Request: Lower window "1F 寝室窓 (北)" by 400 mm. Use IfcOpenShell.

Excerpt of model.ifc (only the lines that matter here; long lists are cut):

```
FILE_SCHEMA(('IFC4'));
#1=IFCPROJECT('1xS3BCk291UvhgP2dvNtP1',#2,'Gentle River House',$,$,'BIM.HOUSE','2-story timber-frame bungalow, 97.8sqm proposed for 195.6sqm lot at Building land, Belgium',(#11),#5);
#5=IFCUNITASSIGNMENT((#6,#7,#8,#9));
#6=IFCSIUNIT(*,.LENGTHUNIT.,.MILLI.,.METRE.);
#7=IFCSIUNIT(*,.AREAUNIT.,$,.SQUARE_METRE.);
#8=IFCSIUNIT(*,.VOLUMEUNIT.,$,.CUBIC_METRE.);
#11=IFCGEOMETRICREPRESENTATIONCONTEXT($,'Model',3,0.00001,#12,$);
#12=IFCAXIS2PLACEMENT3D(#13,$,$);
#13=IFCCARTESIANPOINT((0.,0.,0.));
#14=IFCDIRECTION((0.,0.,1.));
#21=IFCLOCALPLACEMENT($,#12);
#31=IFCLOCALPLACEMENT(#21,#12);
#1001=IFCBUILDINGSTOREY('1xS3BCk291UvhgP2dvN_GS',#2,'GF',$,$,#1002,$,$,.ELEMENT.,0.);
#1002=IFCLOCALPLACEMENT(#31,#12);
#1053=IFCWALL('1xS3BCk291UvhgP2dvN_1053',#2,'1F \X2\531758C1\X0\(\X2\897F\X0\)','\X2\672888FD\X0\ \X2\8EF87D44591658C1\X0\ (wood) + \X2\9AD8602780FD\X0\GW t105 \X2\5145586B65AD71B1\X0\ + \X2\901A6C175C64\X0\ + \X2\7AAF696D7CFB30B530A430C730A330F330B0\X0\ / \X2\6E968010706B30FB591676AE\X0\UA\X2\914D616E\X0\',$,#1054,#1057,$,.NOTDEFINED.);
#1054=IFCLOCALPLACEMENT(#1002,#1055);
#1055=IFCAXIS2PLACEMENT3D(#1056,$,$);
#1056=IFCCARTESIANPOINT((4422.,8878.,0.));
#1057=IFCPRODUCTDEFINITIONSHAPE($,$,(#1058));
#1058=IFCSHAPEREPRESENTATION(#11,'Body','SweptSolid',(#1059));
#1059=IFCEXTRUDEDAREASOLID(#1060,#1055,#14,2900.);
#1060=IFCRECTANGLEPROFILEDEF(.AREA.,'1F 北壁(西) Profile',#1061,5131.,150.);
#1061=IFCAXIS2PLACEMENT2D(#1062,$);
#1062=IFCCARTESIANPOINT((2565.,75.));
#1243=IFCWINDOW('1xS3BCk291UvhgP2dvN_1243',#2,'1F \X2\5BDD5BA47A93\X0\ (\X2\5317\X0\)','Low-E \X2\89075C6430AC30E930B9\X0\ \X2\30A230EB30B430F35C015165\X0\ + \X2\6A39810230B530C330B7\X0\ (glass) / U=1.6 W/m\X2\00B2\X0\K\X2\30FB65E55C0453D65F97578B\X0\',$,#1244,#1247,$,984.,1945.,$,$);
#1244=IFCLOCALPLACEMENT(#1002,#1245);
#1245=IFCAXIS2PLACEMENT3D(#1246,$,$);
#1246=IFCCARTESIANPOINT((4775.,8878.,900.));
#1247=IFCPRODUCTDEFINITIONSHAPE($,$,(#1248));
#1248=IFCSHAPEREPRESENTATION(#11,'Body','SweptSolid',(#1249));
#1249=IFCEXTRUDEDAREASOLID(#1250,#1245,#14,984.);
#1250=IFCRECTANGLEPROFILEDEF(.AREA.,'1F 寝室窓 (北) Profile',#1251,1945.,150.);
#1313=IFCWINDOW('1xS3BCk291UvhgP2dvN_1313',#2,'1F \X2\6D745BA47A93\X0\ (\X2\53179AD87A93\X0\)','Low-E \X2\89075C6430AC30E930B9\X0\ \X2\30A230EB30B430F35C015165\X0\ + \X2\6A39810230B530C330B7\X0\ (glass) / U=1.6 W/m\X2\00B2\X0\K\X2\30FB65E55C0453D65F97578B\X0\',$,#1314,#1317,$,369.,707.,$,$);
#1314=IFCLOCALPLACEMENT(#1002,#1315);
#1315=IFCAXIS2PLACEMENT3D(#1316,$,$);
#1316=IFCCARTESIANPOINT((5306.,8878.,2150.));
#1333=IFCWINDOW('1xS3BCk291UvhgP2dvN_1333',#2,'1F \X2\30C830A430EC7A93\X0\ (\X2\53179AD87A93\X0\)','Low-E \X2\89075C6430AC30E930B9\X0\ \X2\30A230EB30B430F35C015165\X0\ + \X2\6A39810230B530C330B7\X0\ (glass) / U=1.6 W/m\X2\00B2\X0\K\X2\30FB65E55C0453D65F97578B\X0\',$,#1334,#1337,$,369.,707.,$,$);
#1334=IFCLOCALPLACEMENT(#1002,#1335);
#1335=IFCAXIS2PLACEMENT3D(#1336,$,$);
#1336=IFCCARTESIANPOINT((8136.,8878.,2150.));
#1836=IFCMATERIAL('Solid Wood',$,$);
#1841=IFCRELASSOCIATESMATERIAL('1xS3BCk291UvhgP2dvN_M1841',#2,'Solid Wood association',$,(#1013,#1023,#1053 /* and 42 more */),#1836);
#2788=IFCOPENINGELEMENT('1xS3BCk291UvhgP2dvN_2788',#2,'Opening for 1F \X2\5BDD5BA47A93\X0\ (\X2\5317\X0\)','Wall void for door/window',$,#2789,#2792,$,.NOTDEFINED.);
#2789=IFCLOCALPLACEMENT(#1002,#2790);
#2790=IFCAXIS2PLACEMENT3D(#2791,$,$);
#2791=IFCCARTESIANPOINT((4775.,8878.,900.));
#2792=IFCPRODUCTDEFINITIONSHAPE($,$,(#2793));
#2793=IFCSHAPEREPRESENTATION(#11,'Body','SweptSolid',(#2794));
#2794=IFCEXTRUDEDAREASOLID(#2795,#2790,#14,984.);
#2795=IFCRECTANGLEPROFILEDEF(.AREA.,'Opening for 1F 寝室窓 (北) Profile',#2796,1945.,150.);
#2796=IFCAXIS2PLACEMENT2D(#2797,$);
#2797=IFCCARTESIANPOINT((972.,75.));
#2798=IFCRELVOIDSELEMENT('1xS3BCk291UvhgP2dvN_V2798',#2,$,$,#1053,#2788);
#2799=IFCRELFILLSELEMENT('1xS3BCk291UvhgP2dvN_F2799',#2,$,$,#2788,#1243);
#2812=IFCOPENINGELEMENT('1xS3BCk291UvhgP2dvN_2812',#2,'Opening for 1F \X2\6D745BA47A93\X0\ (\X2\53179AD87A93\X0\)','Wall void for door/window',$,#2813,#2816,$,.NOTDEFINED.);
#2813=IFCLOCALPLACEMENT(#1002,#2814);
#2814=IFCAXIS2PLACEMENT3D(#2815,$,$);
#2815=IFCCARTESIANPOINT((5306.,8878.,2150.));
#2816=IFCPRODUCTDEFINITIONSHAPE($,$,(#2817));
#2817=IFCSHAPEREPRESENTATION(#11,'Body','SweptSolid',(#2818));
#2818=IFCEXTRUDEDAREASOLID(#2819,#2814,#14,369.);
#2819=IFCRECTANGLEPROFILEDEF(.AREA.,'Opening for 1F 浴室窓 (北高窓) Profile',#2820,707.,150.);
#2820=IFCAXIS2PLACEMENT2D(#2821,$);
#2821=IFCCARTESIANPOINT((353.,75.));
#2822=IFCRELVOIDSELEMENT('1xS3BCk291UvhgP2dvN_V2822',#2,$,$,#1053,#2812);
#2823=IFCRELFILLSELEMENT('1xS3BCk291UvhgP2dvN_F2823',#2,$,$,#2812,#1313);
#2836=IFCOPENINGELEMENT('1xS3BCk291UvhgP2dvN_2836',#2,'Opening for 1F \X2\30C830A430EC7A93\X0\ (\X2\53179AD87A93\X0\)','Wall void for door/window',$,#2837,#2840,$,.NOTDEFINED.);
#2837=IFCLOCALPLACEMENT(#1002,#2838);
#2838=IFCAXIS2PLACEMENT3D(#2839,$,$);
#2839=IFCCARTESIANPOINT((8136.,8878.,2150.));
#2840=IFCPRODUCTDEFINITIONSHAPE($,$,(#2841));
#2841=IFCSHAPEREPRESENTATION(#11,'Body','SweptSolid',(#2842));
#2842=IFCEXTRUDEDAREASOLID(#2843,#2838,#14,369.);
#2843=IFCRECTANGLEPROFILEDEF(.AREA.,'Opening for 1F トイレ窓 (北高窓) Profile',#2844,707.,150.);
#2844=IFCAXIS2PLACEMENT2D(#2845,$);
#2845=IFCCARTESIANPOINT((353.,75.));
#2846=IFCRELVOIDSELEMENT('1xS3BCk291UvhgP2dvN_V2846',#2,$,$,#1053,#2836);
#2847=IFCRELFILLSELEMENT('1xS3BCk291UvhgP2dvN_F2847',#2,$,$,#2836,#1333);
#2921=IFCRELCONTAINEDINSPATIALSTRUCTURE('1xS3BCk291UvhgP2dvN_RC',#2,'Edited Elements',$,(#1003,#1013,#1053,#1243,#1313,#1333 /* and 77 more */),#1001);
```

```python
import numpy as np
import ifcopenshell
import ifcopenshell.api.geometry
import ifcopenshell.util.placement
import ifcopenshell.util.unit

model = ifcopenshell.open("model.ifc")
unit_scale = ifcopenshell.util.unit.calculate_unit_scale(model)

window = model.by_id(1243)
opening = window.FillsVoids[0].RelatingOpeningElement
dz = -400.0

shift = np.array([0.0, 0.0, dz])
# The window is not placed relative to its opening, so move both.
for product in (opening, window):
    matrix = ifcopenshell.util.placement.get_local_placement(product.ObjectPlacement)
    matrix[:3, 3] += shift
    ifcopenshell.api.geometry.edit_object_placement(model, product=product, matrix=matrix, is_si=False)

print(f"moved by {dz * unit_scale:+.3f} m")

model.write("model_v2.ifc")
```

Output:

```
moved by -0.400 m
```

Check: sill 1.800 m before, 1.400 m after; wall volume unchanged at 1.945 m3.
